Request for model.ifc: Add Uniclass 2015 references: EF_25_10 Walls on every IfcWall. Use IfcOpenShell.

First a look at what the model holds.

```python
import ifcopenshell

model = ifcopenshell.open("model.ifc")
print(model.schema)
print("classifications:", [c.Name for c in model.by_type("IfcClassification")])
for ifc_class in ("IfcDoor", "IfcRoof", "IfcStair", "IfcWall", "IfcWindow"):
    print(ifc_class, len(model.by_type(ifc_class)))
```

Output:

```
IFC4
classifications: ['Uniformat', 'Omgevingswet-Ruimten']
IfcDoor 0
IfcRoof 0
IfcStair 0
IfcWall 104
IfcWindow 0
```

```python
import ifcopenshell
import ifcopenshell.api.classification

model = ifcopenshell.open("model.ifc")

system = ifcopenshell.api.classification.add_classification(model, classification="Uniclass 2015")

codes = {
    "IfcWall": ("EF_25_10", "Walls"),
}
for ifc_class, (code, name) in codes.items():
    products = model.by_type(ifc_class)
    ifcopenshell.api.classification.add_reference(
        model, products=products, classification=system, identification=code, name=name
    )
    print(code, len(products))

model.write("model-out.ifc")
```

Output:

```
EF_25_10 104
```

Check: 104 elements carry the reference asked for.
